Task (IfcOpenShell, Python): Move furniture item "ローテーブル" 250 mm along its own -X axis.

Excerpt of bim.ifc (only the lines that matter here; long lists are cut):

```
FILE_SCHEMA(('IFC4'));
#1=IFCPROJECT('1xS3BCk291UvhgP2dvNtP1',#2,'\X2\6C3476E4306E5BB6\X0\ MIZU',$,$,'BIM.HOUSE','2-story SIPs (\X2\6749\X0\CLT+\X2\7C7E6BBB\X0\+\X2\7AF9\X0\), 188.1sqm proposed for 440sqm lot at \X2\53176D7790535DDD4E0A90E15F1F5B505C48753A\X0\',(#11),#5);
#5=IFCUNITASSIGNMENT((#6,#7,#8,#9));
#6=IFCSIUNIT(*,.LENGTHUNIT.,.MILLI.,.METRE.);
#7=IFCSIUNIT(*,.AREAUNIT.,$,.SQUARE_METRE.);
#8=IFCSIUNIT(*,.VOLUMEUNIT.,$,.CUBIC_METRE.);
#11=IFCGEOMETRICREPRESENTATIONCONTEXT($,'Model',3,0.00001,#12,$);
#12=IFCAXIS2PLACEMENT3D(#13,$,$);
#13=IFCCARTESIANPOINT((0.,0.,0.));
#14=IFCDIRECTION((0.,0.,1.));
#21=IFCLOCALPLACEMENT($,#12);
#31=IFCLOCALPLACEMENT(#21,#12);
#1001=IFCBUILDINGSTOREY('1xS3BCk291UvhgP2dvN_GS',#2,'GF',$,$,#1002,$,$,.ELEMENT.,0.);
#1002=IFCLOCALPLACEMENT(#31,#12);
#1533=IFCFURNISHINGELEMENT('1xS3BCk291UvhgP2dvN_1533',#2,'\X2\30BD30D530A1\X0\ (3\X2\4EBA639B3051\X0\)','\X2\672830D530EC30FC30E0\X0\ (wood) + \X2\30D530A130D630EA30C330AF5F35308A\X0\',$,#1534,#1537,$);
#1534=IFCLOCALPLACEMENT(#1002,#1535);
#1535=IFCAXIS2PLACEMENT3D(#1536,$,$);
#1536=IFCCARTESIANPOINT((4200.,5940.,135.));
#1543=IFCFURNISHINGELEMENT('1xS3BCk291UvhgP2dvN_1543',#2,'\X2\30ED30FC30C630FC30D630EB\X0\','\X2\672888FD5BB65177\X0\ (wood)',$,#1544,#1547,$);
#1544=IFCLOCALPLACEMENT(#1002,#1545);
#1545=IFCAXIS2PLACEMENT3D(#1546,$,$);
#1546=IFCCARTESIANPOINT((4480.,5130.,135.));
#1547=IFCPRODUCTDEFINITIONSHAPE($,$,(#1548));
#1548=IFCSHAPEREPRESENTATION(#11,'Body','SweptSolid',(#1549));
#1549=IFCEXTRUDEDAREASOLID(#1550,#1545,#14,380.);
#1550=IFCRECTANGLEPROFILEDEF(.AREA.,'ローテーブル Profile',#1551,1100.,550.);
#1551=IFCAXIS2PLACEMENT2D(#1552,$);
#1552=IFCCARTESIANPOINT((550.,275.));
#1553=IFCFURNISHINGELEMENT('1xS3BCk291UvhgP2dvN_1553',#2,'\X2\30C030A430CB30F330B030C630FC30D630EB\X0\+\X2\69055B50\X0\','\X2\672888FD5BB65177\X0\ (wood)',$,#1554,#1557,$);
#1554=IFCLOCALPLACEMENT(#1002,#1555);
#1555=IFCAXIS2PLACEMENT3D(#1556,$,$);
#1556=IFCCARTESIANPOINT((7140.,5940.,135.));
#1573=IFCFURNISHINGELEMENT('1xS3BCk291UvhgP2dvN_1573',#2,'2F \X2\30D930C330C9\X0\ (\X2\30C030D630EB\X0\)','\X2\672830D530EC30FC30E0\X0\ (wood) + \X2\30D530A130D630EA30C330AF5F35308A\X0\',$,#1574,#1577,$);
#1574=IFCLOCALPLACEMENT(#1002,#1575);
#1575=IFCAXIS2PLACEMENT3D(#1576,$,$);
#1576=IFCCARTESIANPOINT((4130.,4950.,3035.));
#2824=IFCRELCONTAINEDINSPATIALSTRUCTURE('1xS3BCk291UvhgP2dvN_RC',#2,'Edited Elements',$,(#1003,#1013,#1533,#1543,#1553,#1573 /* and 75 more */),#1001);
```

```python
import ifcopenshell
import ifcopenshell.api.geometry
import ifcopenshell.util.placement

model = ifcopenshell.open("bim.ifc")

item = model.by_guid("1xS3BCk291UvhgP2dvN_1543")
matrix = ifcopenshell.util.placement.get_local_placement(item.ObjectPlacement)
matrix[:3, 3] -= matrix[:3, 0] * 250.0
ifcopenshell.api.geometry.edit_object_placement(model, product=item, matrix=matrix, is_si=False)

print(ifcopenshell.util.placement.get_local_placement(item.ObjectPlacement).round(3) + 0.0)

model.write("bim_rev.ifc")
```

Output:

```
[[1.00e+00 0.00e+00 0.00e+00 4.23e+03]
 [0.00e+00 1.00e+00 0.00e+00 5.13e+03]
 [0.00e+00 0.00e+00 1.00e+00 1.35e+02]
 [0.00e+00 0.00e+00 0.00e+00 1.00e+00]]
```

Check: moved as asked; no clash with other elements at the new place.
